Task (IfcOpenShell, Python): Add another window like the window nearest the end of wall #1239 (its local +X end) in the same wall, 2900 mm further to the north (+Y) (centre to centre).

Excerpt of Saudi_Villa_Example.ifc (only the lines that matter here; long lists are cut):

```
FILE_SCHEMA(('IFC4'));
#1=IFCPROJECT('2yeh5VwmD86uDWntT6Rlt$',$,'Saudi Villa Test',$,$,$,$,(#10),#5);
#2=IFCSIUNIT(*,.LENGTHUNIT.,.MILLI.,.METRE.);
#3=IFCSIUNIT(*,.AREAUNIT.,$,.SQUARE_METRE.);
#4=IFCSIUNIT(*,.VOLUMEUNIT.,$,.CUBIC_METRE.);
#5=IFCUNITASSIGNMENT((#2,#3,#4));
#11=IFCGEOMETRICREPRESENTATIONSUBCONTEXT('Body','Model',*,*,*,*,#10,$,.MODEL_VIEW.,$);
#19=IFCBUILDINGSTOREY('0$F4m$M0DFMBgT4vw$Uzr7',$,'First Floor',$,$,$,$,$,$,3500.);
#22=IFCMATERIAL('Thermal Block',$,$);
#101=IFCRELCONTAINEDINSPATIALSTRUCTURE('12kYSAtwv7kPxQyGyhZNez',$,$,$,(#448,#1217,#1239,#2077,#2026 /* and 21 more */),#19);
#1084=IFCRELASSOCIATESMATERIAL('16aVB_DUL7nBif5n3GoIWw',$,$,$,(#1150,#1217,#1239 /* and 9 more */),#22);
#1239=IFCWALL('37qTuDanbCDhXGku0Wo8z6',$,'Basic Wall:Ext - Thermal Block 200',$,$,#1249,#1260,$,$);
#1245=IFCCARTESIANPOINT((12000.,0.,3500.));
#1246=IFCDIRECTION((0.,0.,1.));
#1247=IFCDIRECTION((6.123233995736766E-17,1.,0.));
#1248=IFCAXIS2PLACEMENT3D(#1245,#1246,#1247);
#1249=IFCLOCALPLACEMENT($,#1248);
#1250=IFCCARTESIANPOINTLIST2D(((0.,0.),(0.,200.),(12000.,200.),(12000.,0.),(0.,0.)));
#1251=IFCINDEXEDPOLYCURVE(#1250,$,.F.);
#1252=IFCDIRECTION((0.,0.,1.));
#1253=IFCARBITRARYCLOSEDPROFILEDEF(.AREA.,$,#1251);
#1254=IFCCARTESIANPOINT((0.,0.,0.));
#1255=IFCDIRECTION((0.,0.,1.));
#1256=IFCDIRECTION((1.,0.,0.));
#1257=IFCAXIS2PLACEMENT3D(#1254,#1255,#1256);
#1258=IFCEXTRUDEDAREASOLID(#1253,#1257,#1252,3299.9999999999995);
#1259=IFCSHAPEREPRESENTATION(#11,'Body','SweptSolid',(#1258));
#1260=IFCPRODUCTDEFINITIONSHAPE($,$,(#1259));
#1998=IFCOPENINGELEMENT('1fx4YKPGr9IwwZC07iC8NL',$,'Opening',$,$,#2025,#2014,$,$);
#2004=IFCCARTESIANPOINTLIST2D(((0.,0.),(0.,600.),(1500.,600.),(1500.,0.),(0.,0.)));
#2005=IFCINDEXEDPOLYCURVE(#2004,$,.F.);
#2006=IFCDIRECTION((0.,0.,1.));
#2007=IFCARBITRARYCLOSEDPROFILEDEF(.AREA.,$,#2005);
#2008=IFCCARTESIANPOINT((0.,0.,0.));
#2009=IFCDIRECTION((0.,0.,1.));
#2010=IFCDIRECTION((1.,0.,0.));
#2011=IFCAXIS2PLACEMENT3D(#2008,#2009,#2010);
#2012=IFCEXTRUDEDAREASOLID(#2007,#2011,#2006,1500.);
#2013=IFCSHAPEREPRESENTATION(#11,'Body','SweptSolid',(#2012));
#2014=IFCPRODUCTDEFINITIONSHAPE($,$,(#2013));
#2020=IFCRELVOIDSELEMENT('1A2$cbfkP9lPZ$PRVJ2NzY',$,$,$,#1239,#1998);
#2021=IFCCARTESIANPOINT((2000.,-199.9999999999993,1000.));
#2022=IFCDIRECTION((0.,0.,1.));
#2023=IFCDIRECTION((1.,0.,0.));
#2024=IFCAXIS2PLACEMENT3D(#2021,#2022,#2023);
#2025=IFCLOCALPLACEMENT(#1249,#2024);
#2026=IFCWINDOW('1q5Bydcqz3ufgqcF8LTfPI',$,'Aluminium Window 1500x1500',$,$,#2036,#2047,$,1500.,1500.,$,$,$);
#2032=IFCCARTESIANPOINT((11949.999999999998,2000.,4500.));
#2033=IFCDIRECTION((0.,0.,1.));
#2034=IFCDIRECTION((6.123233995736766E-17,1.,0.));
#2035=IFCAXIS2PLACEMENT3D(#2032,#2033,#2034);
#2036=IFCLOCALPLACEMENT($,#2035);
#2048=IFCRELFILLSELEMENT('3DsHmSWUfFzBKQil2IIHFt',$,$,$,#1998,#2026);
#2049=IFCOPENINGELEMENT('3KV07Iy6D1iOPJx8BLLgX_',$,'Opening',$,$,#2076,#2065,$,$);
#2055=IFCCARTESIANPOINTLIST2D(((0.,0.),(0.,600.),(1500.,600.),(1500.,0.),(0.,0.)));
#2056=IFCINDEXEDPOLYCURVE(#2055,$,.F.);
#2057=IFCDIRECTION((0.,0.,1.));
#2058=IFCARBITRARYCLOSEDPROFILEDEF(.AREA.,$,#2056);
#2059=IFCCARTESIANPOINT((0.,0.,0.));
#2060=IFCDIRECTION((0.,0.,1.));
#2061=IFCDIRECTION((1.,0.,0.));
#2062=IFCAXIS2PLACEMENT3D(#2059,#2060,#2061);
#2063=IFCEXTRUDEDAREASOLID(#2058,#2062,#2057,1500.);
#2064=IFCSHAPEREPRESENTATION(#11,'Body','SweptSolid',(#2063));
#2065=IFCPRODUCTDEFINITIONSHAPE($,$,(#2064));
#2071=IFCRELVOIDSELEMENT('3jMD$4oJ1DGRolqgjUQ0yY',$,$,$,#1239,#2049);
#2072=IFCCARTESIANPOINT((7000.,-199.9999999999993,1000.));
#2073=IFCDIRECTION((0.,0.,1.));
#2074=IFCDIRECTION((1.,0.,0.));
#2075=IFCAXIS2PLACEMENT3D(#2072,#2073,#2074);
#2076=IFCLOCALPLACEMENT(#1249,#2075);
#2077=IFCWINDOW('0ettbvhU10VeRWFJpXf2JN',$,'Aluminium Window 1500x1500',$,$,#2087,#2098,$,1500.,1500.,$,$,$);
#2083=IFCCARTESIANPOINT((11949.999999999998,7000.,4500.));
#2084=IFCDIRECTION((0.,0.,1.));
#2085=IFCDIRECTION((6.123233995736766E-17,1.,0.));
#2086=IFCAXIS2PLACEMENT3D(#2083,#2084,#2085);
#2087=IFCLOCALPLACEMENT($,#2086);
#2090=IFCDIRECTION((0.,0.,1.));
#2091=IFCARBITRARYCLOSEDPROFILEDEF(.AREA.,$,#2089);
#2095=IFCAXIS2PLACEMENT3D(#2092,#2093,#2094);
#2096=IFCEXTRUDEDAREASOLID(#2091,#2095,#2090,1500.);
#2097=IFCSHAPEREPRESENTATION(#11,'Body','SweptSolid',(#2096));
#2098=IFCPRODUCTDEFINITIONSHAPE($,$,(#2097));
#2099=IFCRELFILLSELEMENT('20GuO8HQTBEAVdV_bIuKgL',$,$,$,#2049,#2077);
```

```python
import ifcopenshell
import ifcopenshell.api.feature
import ifcopenshell.api.geometry
import ifcopenshell.api.root
import ifcopenshell.geom
import ifcopenshell.util.element
import ifcopenshell.util.placement
import ifcopenshell.util.shape
import ifcopenshell.util.unit

model = ifcopenshell.open("Saudi_Villa_Example.ifc")
unit_scale = ifcopenshell.util.unit.calculate_unit_scale(model)
settings = ifcopenshell.geom.settings()


def volume(element):
    """Net volume in cubic metres, openings subtracted."""
    shape = ifcopenshell.geom.create_shape(settings, element)
    return ifcopenshell.util.shape.get_volume(shape.geometry)


window = model.by_guid("0ettbvhU10VeRWFJpXf2JN")
opening = window.FillsVoids[0].RelatingOpeningElement
wall = opening.VoidsElements[0].RelatingBuildingElement
before = volume(wall)
shift = ifcopenshell.util.placement.get_local_placement(wall.ObjectPlacement)[:3, 0] * 2.9 / unit_scale

# copy_class copies the void relationship, type, container and properties, but no geometry.
new_opening = ifcopenshell.api.root.copy_class(model, product=opening)
new_opening.Representation = ifcopenshell.util.element.copy_deep(
    model, opening.Representation, exclude=["IfcGeometricRepresentationContext", "IfcRepresentationMap"]
)
new_window = ifcopenshell.api.root.copy_class(model, product=window)
new_window.Representation = ifcopenshell.util.element.copy_deep(
    model, window.Representation, exclude=["IfcGeometricRepresentationContext", "IfcRepresentationMap"]
)
ifcopenshell.api.feature.add_filling(model, opening=new_opening, element=new_window)

for old, new in ((opening, new_opening), (window, new_window)):
    matrix = ifcopenshell.util.placement.get_local_placement(old.ObjectPlacement)
    matrix[:3, 3] += shift
    ifcopenshell.api.geometry.edit_object_placement(model, product=new, matrix=matrix, is_si=False)

after = volume(wall)

print(f"wall volume {before:.3f} -> {after:.3f} m3")

model.write("Saudi_Villa_Example_v2.ifc")
```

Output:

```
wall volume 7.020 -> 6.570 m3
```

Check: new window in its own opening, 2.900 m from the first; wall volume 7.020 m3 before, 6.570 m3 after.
